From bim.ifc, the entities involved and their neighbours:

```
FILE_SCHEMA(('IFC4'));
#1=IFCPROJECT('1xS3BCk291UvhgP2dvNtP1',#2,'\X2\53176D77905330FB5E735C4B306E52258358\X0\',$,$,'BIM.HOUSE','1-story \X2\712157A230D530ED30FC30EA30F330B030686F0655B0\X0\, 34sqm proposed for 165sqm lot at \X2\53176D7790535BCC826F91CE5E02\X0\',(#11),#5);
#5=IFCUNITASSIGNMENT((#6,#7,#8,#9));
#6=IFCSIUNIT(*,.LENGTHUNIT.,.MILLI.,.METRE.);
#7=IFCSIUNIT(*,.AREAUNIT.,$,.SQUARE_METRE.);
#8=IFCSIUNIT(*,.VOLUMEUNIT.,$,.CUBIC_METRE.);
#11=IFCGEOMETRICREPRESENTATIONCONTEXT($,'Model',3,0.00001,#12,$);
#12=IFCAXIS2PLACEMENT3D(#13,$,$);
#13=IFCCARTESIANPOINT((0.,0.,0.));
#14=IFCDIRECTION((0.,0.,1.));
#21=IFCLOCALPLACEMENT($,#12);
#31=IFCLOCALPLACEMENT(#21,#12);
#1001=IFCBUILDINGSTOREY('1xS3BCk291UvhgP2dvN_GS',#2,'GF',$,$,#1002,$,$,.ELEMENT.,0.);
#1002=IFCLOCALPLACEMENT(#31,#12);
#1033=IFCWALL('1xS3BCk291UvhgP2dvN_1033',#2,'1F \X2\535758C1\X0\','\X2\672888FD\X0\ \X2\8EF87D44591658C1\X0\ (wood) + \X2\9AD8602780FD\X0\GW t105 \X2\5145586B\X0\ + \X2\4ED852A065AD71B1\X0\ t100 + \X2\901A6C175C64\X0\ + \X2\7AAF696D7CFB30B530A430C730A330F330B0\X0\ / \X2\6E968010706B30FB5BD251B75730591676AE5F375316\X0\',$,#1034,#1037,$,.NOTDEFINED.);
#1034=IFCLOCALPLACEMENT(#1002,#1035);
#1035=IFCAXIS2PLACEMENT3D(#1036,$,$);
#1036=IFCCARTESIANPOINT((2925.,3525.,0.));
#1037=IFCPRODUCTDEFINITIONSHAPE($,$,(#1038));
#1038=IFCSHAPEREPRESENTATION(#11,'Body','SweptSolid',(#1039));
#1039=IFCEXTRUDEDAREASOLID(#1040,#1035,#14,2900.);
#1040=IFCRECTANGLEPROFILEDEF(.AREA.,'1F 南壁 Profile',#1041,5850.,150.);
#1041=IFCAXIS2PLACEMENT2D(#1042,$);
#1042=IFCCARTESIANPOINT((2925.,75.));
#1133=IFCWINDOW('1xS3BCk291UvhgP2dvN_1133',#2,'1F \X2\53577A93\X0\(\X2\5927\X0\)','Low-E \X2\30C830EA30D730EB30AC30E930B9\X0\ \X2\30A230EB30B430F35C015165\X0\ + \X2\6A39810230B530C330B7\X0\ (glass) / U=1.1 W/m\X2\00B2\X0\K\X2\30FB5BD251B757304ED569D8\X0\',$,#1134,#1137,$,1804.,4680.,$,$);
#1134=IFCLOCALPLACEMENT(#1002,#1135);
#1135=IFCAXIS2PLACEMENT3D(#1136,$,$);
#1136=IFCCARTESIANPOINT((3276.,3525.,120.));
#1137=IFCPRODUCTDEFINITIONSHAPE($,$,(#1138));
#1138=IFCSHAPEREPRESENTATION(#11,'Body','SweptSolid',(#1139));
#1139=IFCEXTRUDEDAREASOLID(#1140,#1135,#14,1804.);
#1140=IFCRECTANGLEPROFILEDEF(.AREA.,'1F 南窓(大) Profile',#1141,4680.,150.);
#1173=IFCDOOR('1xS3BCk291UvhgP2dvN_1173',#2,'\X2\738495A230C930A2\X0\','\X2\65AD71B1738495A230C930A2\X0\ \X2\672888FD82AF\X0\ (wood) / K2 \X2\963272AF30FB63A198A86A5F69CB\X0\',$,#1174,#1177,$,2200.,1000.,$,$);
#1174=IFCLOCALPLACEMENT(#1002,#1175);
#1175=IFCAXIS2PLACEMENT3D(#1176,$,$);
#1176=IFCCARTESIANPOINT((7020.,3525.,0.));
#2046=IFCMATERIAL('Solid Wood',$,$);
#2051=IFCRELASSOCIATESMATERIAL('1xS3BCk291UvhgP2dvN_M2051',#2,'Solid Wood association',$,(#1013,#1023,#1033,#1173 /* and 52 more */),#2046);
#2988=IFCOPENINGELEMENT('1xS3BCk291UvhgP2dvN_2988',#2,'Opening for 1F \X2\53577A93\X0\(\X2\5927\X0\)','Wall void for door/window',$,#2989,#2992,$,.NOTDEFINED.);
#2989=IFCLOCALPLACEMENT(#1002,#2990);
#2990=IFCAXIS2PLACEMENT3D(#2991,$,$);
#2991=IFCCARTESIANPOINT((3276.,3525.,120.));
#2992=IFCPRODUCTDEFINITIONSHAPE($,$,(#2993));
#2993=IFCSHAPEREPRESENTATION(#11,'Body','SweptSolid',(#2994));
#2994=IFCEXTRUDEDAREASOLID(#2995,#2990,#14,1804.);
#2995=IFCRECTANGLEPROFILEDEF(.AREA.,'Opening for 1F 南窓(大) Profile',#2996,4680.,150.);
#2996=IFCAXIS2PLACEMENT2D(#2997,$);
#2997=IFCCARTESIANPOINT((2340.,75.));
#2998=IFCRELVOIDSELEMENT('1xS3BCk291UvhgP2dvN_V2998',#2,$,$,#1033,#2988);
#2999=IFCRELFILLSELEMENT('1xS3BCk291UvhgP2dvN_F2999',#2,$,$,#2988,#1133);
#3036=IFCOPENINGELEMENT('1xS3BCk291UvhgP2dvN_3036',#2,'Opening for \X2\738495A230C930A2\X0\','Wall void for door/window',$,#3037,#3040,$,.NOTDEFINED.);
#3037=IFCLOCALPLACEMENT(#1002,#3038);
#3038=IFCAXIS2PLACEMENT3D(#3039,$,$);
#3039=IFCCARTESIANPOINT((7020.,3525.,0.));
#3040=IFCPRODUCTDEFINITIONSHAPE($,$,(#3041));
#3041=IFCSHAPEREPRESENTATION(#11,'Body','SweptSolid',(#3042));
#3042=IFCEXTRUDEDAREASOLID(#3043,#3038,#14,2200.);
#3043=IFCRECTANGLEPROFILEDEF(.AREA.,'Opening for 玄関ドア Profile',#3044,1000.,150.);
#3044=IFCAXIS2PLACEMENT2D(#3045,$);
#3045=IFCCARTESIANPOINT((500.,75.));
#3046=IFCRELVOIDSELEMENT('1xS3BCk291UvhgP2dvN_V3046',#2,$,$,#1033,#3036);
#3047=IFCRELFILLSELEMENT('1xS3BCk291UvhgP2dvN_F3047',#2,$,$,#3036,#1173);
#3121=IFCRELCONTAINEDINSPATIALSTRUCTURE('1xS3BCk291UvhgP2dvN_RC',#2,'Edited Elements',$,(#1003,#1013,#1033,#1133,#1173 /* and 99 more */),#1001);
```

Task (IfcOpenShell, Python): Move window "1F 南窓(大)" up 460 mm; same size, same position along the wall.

```python
import numpy as np
import ifcopenshell
import ifcopenshell.api.geometry
import ifcopenshell.util.placement
import ifcopenshell.util.unit

model = ifcopenshell.open("bim.ifc")
unit_scale = ifcopenshell.util.unit.calculate_unit_scale(model)

window = model.by_id(1133)
opening = window.FillsVoids[0].RelatingOpeningElement
dz = 460.0

shift = np.array([0.0, 0.0, dz])
# The window is not placed relative to its opening, so move both.
for product in (opening, window):
    matrix = ifcopenshell.util.placement.get_local_placement(product.ObjectPlacement)
    matrix[:3, 3] += shift
    ifcopenshell.api.geometry.edit_object_placement(model, product=product, matrix=matrix, is_si=False)

print(f"moved by {dz * unit_scale:+.3f} m")

model.write("bim-out.ifc")
```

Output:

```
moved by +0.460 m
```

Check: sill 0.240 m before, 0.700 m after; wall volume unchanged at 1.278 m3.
